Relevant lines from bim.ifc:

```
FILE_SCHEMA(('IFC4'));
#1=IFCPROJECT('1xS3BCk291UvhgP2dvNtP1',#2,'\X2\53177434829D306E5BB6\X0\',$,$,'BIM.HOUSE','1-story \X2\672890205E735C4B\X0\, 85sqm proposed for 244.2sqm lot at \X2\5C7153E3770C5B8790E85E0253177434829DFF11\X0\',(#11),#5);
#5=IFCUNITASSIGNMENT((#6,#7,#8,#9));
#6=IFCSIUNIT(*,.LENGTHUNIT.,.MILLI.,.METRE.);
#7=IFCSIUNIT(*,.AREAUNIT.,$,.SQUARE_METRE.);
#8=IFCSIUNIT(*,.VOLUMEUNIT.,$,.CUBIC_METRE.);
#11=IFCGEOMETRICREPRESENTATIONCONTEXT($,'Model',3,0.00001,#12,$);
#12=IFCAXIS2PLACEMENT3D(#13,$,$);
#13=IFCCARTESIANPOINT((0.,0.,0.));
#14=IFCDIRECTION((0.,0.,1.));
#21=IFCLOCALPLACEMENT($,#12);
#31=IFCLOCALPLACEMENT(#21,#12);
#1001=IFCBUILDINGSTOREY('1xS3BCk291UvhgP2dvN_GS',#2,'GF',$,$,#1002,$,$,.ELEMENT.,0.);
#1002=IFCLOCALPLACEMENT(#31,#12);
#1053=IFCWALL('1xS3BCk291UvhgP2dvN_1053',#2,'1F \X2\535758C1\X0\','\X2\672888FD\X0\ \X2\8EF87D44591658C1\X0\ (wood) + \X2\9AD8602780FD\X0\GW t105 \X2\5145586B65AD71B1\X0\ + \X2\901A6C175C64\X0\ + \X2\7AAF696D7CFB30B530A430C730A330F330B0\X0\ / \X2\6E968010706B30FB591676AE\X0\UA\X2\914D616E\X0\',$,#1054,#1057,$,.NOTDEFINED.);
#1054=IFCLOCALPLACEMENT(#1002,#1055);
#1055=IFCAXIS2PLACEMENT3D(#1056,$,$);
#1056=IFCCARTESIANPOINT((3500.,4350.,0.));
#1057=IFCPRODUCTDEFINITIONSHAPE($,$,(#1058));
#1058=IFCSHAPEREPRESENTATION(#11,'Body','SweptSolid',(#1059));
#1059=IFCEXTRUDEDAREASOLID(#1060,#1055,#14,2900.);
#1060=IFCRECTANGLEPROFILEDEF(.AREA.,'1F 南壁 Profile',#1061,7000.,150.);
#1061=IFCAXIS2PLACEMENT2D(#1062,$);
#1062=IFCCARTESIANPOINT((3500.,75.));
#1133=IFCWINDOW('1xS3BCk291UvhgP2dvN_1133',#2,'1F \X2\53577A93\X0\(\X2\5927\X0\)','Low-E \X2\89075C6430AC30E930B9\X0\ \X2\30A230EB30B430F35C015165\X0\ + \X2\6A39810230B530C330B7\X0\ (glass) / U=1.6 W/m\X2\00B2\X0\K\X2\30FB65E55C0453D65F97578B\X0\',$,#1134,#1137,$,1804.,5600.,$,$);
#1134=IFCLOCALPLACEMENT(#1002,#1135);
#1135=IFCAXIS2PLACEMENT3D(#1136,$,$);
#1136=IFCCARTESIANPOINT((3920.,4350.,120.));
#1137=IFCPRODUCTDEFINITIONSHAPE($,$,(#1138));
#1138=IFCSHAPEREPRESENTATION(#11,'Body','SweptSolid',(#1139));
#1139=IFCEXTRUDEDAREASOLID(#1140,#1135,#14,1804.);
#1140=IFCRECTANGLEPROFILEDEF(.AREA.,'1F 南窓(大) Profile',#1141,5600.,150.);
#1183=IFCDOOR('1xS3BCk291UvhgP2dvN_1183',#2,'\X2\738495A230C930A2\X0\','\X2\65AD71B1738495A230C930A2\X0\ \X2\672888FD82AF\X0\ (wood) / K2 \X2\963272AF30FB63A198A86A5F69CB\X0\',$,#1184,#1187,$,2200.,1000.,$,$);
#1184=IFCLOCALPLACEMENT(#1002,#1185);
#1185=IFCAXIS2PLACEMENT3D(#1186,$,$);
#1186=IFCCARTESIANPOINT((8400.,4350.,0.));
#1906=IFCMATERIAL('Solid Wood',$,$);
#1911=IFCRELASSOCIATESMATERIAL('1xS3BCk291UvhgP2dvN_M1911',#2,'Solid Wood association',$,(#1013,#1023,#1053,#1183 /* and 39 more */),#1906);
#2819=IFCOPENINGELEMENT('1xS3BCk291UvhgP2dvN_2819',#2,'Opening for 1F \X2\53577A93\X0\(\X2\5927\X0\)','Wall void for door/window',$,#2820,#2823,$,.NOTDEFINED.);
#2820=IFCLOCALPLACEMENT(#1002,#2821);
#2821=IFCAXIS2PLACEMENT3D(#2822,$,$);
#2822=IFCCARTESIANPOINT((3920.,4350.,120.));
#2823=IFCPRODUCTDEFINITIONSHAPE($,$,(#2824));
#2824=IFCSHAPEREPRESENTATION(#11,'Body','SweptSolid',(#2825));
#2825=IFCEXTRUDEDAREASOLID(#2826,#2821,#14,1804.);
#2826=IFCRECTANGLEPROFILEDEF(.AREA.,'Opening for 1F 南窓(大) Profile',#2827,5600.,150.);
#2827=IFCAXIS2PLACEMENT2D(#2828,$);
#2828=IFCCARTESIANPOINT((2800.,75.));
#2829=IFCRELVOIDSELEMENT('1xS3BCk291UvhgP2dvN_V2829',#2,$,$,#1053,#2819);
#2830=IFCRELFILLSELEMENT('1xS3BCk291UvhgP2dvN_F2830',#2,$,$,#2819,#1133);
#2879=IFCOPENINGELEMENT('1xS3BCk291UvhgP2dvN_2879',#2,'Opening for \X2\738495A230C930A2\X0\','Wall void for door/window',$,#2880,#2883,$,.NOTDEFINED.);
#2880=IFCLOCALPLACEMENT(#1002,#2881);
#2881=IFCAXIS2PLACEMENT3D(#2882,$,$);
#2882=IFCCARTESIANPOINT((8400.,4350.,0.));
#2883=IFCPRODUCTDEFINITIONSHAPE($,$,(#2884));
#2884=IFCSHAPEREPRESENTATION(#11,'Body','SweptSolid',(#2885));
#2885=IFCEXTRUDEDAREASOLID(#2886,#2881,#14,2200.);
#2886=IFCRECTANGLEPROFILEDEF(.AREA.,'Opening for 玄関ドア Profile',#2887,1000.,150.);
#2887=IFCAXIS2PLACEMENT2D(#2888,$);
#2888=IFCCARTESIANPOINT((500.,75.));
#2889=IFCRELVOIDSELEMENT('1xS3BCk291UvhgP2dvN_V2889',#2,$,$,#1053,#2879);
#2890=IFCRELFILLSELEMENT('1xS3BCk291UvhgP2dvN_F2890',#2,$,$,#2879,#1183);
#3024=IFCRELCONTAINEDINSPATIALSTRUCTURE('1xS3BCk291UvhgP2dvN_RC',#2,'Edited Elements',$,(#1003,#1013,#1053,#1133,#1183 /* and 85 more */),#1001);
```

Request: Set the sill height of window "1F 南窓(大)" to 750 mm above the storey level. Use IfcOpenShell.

```python
import numpy as np
import ifcopenshell
import ifcopenshell.api.geometry
import ifcopenshell.geom
import ifcopenshell.util.element
import ifcopenshell.util.placement
import ifcopenshell.util.shape
import ifcopenshell.util.unit

model = ifcopenshell.open("bim.ifc")
unit_scale = ifcopenshell.util.unit.calculate_unit_scale(model)

window = model.by_guid("1xS3BCk291UvhgP2dvN_1133")
opening = window.FillsVoids[0].RelatingOpeningElement
storey = ifcopenshell.util.element.get_container(window, ifc_class="IfcBuildingStorey")
level = ifcopenshell.util.placement.get_local_placement(storey.ObjectPlacement)[2, 3]

# The opening's origin need not be at the sill, so measure its lowest point.
shape = ifcopenshell.geom.create_shape(ifcopenshell.geom.settings(), opening)
bottom = ifcopenshell.util.shape.get_shape_bottom_elevation(shape, shape.geometry) / unit_scale
dz = level + 0.75 / unit_scale - bottom

shift = np.array([0.0, 0.0, dz])
# The window is not placed relative to its opening, so move both.
for product in (opening, window):
    matrix = ifcopenshell.util.placement.get_local_placement(product.ObjectPlacement)
    matrix[:3, 3] += shift
    ifcopenshell.api.geometry.edit_object_placement(model, product=product, matrix=matrix, is_si=False)

print(f"moved by {dz * unit_scale:+.3f} m")

model.write("bim_rev.ifc")
```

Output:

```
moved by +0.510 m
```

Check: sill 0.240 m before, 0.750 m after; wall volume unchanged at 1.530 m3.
